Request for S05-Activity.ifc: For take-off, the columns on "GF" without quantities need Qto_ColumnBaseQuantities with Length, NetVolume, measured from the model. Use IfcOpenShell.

First a look at what the model holds.

```python
import ifcopenshell
import ifcopenshell.util.element
import ifcopenshell.util.unit

model = ifcopenshell.open("S05-Activity.ifc")
print(model.schema)
for unit_type in ("LENGTHUNIT", "AREAUNIT", "VOLUMEUNIT"):
    print(unit_type, ifcopenshell.util.unit.calculate_unit_scale(model, unit_type))
storey = next(s for s in model.by_type("IfcBuildingStorey") if s.Name == "GF")
columns = [e for e in ifcopenshell.util.element.get_decomposition(storey) if e.is_a("IfcColumn")]
for e in sorted(columns, key=lambda e: e.id()):
    print(e.id(), e.is_a(), e.Name, list(ifcopenshell.util.element.get_psets(e, qtos_only=True)), sep=" | ")
```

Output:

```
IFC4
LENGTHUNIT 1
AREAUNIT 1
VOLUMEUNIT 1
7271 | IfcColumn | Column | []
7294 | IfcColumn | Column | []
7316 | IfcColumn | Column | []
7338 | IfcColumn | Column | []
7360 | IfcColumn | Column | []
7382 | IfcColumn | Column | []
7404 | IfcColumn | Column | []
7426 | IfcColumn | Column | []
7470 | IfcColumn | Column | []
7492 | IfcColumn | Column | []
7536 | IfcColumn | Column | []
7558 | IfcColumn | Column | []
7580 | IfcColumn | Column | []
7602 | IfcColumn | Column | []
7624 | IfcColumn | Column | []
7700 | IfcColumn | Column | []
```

```python
import ifcopenshell
import ifcopenshell.api.pset
import ifcopenshell.geom
import ifcopenshell.util.element
import ifcopenshell.util.shape
import ifcopenshell.util.unit

model = ifcopenshell.open("S05-Activity.ifc")
unit_scale = ifcopenshell.util.unit.calculate_unit_scale(model)
volume_scale = ifcopenshell.util.unit.calculate_unit_scale(model, "VOLUMEUNIT")
settings = ifcopenshell.geom.settings()

storey = next(s for s in model.by_type("IfcBuildingStorey") if s.Name == "GF")
columns = [e for e in ifcopenshell.util.element.get_decomposition(storey) if e.is_a("IfcColumn")]

for e in sorted(columns, key=lambda e: e.id()):
    if ifcopenshell.util.element.get_psets(e, qtos_only=True, should_inherit=False):
        continue
    # Geometry comes back in metres, in the element's own axes.
    shape = ifcopenshell.geom.create_shape(settings, e)
    values = {
        "Length": ifcopenshell.util.shape.get_z(shape.geometry) / unit_scale,
        "NetVolume": ifcopenshell.util.shape.get_volume(shape.geometry) / volume_scale,
    }
    qto = ifcopenshell.api.pset.add_qto(model, product=e, name="Qto_ColumnBaseQuantities")
    ifcopenshell.api.pset.edit_qto(model, qto=qto, properties=values)
    print(e.id(), {k: round(v, 3) for k, v in values.items()})

model.write("S05-Activity_rev.ifc")
```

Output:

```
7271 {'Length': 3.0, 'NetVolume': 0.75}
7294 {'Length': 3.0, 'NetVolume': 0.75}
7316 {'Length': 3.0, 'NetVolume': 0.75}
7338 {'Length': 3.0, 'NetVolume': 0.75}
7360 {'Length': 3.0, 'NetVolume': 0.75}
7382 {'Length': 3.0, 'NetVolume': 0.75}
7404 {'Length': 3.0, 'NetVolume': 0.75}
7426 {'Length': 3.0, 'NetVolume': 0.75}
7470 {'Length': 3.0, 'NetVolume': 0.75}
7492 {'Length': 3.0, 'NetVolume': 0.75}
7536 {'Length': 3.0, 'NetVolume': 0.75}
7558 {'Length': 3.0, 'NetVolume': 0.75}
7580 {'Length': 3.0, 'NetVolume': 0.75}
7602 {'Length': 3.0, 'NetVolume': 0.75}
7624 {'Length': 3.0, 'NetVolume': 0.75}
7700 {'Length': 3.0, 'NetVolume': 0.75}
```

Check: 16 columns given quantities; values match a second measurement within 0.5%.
